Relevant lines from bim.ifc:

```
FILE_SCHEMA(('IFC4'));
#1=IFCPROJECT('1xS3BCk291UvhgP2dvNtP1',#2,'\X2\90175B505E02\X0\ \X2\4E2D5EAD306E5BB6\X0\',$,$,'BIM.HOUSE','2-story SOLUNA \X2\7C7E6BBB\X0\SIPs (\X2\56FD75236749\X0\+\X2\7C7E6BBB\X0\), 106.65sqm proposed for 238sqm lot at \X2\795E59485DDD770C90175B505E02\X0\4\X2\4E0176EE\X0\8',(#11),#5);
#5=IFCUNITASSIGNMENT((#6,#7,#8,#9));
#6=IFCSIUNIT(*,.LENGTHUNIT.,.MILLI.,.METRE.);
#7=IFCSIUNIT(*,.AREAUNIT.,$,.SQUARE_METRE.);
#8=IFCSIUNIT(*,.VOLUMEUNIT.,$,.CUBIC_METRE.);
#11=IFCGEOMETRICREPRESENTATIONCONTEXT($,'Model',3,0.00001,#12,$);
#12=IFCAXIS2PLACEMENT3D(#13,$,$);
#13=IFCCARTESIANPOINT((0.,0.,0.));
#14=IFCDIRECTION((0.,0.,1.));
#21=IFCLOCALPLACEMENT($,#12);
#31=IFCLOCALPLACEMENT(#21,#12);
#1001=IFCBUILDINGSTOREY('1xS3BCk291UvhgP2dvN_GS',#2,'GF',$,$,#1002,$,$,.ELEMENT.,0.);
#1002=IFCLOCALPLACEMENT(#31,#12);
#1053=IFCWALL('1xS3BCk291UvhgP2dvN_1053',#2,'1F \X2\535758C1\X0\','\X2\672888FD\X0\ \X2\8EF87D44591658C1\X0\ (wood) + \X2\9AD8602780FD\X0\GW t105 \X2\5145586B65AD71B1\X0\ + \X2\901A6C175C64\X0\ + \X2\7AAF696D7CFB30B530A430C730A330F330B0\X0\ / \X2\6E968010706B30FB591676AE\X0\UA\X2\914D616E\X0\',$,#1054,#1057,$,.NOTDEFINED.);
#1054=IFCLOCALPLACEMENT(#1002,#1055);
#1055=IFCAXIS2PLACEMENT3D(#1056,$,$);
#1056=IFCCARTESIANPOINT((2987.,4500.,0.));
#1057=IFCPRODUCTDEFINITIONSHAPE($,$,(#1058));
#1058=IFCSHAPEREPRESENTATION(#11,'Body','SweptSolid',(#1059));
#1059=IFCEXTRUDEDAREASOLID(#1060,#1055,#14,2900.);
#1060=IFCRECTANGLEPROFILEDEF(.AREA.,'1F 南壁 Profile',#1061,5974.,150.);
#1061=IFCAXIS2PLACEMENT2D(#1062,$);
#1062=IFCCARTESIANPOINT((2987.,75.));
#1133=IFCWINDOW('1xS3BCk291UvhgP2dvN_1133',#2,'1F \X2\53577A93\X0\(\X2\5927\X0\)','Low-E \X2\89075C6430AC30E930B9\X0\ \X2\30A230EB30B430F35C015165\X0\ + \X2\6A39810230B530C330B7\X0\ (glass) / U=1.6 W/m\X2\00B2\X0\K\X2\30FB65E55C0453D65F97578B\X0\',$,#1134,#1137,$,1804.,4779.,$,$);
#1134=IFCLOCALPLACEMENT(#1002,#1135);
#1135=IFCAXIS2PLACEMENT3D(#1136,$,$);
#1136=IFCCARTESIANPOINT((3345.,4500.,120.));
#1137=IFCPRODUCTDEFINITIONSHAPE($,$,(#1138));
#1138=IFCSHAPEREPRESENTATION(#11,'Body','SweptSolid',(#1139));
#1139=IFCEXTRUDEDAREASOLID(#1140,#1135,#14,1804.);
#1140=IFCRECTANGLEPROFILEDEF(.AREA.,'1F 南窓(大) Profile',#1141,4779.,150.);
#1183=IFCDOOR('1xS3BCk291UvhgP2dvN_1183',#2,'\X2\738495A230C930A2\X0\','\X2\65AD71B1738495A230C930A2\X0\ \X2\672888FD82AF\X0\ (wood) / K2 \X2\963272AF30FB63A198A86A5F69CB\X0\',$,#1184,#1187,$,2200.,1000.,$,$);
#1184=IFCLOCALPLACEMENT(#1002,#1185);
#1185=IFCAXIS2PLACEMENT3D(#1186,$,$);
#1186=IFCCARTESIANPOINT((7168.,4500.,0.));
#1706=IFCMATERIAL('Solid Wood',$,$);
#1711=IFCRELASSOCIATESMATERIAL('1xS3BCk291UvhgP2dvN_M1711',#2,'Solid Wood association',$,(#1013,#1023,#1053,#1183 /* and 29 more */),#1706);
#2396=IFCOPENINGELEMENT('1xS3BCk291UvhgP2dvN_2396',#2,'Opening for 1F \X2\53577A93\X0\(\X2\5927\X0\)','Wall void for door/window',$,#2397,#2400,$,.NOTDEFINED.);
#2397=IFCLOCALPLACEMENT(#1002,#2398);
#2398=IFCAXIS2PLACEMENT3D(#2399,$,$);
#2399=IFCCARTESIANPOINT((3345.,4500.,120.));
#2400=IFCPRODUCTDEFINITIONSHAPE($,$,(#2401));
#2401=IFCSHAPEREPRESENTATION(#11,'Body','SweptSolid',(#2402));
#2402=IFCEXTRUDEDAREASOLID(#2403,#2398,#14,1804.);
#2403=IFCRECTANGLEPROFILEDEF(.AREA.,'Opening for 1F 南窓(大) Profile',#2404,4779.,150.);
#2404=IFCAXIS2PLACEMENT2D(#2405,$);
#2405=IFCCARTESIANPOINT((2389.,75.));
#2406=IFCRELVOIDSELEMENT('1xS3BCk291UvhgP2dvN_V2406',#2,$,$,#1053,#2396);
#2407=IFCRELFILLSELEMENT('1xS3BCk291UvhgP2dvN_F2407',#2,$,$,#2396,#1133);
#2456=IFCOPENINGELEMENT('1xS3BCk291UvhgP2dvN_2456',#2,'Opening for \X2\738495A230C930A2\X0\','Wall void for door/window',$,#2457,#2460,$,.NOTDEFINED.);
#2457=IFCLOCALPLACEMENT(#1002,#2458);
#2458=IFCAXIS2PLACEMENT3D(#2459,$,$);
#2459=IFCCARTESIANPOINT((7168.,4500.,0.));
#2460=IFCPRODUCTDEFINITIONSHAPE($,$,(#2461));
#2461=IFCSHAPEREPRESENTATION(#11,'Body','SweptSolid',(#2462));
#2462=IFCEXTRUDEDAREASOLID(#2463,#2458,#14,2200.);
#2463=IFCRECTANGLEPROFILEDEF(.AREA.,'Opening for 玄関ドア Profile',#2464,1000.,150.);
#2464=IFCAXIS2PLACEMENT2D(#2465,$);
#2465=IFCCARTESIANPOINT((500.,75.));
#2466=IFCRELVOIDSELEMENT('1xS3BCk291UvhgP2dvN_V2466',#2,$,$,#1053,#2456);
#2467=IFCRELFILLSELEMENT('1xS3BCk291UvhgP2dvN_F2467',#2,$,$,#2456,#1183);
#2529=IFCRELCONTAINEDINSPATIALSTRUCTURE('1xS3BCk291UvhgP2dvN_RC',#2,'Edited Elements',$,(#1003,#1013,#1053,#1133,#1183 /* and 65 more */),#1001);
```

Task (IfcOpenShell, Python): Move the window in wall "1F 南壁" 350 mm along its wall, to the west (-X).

```python
import ifcopenshell
import ifcopenshell.api.geometry
import ifcopenshell.util.placement

model = ifcopenshell.open("bim.ifc")

window = model.by_id(1133)
opening = window.FillsVoids[0].RelatingOpeningElement
wall = opening.VoidsElements[0].RelatingBuildingElement

wall_matrix = ifcopenshell.util.placement.get_local_placement(wall.ObjectPlacement)
shift = wall_matrix[:3, 0] * -350.0
before = ifcopenshell.util.placement.get_local_placement(window.ObjectPlacement)[:3, 3].copy()

# The window is not placed relative to its opening, so move both.
for product in (opening, window):
    matrix = ifcopenshell.util.placement.get_local_placement(product.ObjectPlacement)
    matrix[:3, 3] += shift
    ifcopenshell.api.geometry.edit_object_placement(model, product=product, matrix=matrix, is_si=False)

after = ifcopenshell.util.placement.get_local_placement(window.ObjectPlacement)[:3, 3]
print("window moved by", (after - before).round(3) + 0.0)

model.write("bim_rev.ifc")
```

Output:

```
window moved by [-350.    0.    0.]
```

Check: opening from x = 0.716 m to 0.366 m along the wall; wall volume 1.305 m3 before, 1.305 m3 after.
